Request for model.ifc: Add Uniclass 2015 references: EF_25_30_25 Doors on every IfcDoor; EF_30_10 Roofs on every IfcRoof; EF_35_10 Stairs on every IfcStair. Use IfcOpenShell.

First a look at what the model holds.

```python
import ifcopenshell

model = ifcopenshell.open("model.ifc")
print(model.schema)
print("classifications:", [c.Name for c in model.by_type("IfcClassification")])
for ifc_class in ("IfcDoor", "IfcRoof", "IfcStair", "IfcWall", "IfcWindow"):
    print(ifc_class, len(model.by_type(ifc_class)))
```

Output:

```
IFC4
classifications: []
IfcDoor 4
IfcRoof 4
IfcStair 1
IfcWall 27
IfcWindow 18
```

```python
import ifcopenshell
import ifcopenshell.api.classification

model = ifcopenshell.open("model.ifc")

system = ifcopenshell.api.classification.add_classification(model, classification="Uniclass 2015")

codes = {
    "IfcDoor": ("EF_25_30_25", "Doors"),
    "IfcRoof": ("EF_30_10", "Roofs"),
    "IfcStair": ("EF_35_10", "Stairs"),
}
for ifc_class, (code, name) in codes.items():
    products = model.by_type(ifc_class)
    ifcopenshell.api.classification.add_reference(
        model, products=products, classification=system, identification=code, name=name
    )
    print(code, len(products))

model.write("model_edited.ifc")
```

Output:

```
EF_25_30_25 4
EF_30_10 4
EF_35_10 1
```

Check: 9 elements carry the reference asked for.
